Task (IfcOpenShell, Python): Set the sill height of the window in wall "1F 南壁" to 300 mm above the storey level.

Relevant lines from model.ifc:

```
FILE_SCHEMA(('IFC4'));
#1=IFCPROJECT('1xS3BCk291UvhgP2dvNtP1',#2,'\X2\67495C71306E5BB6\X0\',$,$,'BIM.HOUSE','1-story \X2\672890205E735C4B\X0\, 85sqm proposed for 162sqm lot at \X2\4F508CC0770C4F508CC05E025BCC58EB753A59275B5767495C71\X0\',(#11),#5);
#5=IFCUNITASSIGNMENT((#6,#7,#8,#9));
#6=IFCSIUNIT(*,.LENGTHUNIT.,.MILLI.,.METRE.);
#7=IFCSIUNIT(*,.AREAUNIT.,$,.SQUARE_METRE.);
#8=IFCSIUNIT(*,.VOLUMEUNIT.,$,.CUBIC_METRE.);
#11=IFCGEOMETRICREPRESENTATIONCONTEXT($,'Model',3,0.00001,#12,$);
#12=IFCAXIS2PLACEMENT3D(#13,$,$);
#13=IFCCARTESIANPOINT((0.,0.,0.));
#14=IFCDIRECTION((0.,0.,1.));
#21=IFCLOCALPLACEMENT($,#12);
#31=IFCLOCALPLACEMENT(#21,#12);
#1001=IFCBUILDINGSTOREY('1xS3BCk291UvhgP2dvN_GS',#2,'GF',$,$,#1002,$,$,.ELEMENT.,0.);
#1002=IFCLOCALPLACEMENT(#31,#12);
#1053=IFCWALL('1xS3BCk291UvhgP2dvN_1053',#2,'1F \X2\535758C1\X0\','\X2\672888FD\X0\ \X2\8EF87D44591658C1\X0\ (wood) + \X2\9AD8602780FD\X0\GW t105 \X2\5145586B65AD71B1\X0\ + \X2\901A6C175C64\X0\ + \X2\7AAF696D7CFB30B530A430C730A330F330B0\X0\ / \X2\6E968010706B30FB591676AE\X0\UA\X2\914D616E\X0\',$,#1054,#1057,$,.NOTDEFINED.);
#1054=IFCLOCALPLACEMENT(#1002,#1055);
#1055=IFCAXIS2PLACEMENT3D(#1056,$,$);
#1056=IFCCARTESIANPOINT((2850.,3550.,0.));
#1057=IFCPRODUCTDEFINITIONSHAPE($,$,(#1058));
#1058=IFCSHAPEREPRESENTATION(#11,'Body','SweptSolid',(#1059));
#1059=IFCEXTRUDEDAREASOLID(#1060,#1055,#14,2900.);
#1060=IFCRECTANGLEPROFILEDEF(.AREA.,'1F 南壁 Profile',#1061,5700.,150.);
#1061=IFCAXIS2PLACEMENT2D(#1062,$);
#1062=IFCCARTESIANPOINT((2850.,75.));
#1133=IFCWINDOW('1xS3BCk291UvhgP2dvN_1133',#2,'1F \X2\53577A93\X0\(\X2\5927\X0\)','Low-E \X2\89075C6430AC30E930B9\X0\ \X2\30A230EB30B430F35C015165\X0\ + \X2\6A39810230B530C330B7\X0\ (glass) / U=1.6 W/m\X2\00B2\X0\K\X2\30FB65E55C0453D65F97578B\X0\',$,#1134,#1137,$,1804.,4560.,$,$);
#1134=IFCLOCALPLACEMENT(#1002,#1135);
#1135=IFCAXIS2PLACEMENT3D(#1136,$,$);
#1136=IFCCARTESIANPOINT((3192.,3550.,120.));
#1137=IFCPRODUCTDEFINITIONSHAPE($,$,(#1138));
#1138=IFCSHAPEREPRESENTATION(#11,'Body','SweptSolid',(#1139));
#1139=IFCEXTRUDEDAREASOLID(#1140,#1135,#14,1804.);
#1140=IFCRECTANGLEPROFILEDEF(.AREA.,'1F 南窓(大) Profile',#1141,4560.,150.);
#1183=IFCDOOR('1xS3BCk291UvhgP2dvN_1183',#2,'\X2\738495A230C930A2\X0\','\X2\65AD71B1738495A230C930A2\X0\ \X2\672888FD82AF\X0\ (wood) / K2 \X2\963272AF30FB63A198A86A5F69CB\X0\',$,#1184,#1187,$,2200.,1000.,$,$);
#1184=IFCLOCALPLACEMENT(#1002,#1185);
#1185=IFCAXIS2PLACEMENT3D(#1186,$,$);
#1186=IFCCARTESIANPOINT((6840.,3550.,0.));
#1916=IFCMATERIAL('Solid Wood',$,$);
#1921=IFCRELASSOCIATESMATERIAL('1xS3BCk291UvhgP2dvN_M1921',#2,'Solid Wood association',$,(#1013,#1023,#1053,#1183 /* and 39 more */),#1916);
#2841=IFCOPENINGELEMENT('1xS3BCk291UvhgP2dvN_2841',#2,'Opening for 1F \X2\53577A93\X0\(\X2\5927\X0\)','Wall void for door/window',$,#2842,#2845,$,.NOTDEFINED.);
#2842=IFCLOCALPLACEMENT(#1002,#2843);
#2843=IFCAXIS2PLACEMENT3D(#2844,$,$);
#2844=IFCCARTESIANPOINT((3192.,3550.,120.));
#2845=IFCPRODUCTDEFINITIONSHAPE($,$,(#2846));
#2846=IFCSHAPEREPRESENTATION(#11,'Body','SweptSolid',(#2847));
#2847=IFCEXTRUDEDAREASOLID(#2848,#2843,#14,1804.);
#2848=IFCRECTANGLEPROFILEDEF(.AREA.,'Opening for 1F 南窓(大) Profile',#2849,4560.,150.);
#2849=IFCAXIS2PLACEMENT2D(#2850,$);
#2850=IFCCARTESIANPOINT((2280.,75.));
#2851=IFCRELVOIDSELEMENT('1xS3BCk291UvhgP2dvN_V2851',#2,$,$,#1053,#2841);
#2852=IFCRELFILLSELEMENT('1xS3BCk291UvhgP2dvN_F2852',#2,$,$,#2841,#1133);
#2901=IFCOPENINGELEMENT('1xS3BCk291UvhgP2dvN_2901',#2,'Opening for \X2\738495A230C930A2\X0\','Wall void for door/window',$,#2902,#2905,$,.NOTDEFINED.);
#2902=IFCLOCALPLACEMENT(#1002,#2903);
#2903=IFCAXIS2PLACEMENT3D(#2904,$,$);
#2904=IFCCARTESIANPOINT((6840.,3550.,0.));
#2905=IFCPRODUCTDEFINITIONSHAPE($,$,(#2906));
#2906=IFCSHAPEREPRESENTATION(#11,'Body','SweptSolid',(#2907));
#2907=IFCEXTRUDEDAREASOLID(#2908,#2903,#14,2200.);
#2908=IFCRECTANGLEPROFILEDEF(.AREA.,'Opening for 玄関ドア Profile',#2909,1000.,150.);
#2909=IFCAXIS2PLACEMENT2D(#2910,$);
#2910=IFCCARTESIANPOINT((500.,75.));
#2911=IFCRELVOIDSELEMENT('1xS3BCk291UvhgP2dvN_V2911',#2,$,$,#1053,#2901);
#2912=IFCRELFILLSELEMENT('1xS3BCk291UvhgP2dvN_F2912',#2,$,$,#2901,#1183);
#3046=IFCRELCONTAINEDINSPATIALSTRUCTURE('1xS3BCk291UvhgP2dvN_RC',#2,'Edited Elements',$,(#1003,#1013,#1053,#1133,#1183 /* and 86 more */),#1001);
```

```python
import numpy as np
import ifcopenshell
import ifcopenshell.api.geometry
import ifcopenshell.geom
import ifcopenshell.util.element
import ifcopenshell.util.placement
import ifcopenshell.util.shape
import ifcopenshell.util.unit

model = ifcopenshell.open("model.ifc")
unit_scale = ifcopenshell.util.unit.calculate_unit_scale(model)

window = model.by_id(1133)
opening = window.FillsVoids[0].RelatingOpeningElement
storey = ifcopenshell.util.element.get_container(window, ifc_class="IfcBuildingStorey")
level = ifcopenshell.util.placement.get_local_placement(storey.ObjectPlacement)[2, 3]

# The opening's origin need not be at the sill, so measure its lowest point.
shape = ifcopenshell.geom.create_shape(ifcopenshell.geom.settings(), opening)
bottom = ifcopenshell.util.shape.get_shape_bottom_elevation(shape, shape.geometry) / unit_scale
dz = level + 0.3 / unit_scale - bottom

shift = np.array([0.0, 0.0, dz])
# The window is not placed relative to its opening, so move both.
for product in (opening, window):
    matrix = ifcopenshell.util.placement.get_local_placement(product.ObjectPlacement)
    matrix[:3, 3] += shift
    ifcopenshell.api.geometry.edit_object_placement(model, product=product, matrix=matrix, is_si=False)

print(f"moved by {dz * unit_scale:+.3f} m")

model.write("model_rev.ifc")
```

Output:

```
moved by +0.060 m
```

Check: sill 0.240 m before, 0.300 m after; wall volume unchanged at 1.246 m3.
